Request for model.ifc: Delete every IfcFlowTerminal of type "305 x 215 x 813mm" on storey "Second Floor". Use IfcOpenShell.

First a look at what the model holds.

```python
import ifcopenshell
import ifcopenshell.util.element

model = ifcopenshell.open("model.ifc")
print(model.schema)
storey = next(s for s in model.by_type("IfcBuildingStorey") if s.Name == "Second Floor")
terminals = [e for e in ifcopenshell.util.element.get_decomposition(storey) if e.is_a("IfcFlowTerminal")]
seen = {}
for e in terminals:
    element_type = ifcopenshell.util.element.get_type(e)
    name = element_type.Name if element_type not in (None, e) else None
    seen[name] = seen.get(name, 0) + 1
for name, count in sorted(seen.items(), key=str):
    print(count, "x", name)
```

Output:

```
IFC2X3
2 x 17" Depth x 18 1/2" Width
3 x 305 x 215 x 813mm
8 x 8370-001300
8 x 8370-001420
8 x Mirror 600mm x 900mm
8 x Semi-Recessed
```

```python
import ifcopenshell
import ifcopenshell.api.root
import ifcopenshell.util.element

model = ifcopenshell.open("model.ifc")

storey = next(s for s in model.by_type("IfcBuildingStorey") if s.Name == "Second Floor")
terminals = [e for e in ifcopenshell.util.element.get_decomposition(storey) if e.is_a("IfcFlowTerminal")]
targets = [e for e in terminals if (t := ifcopenshell.util.element.get_type(e)) not in (None, e) and t.Name == "305 x 215 x 813mm"]

for e in targets:
    ifcopenshell.api.root.remove_product(model, product=e)
print(len(targets), "removed")

model.write("model_updated.ifc")
```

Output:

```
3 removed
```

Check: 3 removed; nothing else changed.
